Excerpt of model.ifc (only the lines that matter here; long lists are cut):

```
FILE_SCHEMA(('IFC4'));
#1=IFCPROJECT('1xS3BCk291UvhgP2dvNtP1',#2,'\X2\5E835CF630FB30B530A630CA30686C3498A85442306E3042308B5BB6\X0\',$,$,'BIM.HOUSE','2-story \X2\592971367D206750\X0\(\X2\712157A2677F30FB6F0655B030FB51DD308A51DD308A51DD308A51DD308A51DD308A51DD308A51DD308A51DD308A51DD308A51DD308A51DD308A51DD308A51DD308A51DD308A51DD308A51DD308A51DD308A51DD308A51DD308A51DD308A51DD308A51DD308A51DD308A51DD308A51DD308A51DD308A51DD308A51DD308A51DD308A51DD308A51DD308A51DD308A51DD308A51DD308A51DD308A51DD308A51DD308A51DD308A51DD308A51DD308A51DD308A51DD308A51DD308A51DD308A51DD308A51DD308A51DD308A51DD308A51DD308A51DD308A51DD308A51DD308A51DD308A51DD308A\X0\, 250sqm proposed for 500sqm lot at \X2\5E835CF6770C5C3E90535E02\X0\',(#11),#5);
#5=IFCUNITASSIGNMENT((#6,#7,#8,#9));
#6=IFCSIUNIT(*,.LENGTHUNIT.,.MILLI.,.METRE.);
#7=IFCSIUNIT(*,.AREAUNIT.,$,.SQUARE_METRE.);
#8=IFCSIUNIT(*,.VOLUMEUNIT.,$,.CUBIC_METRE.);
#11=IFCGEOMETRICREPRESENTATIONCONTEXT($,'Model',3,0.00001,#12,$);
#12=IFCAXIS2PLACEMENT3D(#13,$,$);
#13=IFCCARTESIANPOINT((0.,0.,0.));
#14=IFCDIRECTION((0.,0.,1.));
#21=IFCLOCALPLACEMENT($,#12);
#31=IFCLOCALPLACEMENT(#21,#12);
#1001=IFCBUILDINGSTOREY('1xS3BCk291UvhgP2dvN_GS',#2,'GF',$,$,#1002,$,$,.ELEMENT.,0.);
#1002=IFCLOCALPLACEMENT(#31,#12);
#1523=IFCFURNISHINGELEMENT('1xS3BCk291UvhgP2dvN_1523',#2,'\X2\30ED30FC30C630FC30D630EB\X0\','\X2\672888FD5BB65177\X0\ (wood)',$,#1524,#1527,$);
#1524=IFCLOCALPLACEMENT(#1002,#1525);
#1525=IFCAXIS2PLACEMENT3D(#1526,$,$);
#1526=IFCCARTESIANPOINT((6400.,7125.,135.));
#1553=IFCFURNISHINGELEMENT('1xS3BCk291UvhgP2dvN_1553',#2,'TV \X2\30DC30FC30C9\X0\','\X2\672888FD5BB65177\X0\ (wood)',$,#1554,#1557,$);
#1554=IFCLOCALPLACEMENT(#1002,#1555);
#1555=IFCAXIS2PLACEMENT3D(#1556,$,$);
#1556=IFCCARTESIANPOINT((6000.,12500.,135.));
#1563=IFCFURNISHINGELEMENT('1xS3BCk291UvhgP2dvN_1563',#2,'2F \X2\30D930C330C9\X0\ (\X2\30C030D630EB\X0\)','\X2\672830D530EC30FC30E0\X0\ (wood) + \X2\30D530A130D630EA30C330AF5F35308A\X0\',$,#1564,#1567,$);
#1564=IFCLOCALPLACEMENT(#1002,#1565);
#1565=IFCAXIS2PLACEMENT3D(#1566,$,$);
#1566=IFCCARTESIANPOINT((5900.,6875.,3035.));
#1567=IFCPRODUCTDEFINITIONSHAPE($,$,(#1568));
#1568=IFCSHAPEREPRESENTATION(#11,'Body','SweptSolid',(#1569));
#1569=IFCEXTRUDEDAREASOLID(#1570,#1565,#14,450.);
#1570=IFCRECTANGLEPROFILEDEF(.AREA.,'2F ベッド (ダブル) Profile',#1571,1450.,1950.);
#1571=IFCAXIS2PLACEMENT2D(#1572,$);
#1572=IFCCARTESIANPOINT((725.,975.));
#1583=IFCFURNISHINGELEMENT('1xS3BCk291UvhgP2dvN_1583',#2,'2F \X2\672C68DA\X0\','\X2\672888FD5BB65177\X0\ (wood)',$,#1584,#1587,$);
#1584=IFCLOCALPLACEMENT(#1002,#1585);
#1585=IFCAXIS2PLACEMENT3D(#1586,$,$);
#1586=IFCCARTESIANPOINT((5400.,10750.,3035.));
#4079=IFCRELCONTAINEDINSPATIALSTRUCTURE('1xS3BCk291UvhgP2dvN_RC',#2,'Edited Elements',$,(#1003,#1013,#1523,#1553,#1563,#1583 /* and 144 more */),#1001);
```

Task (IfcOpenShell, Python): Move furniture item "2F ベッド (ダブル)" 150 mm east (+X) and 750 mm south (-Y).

```python
import ifcopenshell
import ifcopenshell.api.geometry
import ifcopenshell.util.placement

model = ifcopenshell.open("model.ifc")

item = model.by_guid("1xS3BCk291UvhgP2dvN_1563")
matrix = ifcopenshell.util.placement.get_local_placement(item.ObjectPlacement)
matrix[0, 3] += 150.0
matrix[1, 3] -= 750.0
ifcopenshell.api.geometry.edit_object_placement(model, product=item, matrix=matrix, is_si=False)

print(ifcopenshell.util.placement.get_local_placement(item.ObjectPlacement).round(3) + 0.0)

model.write("model-out.ifc")
```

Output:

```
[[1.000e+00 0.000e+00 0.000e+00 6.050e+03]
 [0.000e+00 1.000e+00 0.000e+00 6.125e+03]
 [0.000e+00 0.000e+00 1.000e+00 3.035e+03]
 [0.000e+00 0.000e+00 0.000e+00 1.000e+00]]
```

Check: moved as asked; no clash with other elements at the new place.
